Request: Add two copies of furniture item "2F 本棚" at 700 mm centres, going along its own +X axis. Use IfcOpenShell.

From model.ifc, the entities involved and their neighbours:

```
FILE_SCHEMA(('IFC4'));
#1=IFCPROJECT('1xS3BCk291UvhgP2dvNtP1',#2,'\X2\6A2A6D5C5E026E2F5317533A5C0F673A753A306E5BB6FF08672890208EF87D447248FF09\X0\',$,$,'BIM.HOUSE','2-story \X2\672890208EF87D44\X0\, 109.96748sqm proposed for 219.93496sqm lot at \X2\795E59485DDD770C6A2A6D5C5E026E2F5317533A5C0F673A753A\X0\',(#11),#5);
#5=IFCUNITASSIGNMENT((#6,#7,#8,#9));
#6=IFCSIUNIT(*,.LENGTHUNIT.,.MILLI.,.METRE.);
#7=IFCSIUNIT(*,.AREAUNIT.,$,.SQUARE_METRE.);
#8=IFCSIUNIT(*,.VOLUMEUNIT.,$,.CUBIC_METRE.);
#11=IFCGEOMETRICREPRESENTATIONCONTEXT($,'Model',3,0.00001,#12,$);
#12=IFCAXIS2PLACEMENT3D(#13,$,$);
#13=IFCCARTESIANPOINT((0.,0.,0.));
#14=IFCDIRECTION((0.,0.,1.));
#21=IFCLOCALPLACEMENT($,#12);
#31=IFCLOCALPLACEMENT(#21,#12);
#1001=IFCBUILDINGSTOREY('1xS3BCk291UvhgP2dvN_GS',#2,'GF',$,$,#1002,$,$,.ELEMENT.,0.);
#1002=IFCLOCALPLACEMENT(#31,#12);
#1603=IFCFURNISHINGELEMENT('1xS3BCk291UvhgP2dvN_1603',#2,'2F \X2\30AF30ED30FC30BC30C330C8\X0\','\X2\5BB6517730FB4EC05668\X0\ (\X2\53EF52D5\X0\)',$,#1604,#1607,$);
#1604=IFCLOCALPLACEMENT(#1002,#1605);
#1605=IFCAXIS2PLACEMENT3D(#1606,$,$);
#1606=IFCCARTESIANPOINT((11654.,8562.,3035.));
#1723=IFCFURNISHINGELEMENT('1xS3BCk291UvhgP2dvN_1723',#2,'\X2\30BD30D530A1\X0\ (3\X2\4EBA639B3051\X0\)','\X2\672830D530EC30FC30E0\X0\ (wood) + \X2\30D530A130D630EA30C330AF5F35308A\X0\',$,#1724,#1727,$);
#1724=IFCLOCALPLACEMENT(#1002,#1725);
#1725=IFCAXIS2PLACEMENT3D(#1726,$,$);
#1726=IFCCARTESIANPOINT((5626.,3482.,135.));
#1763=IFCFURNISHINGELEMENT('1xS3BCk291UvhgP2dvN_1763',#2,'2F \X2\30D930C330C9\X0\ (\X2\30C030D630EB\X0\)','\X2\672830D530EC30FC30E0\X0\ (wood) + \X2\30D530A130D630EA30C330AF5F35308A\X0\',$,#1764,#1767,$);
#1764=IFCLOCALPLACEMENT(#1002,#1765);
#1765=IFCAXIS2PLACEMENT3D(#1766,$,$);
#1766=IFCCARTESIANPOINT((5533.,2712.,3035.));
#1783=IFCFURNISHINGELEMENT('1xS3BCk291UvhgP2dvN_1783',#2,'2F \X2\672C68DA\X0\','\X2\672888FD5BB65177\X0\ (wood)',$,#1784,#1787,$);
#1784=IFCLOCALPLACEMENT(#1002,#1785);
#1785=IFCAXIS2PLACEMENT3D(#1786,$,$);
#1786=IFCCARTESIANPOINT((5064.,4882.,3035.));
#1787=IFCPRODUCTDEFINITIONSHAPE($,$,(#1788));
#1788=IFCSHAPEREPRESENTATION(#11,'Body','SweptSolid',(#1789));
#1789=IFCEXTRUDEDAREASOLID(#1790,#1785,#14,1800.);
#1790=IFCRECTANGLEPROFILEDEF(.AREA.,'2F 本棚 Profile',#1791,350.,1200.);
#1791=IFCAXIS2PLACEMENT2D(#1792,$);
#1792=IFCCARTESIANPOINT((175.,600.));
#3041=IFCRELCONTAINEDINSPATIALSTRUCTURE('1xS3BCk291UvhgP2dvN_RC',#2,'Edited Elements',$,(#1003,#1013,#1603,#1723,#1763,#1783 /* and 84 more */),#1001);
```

```python
import ifcopenshell
import ifcopenshell.api.geometry
import ifcopenshell.api.root
import ifcopenshell.util.element
import ifcopenshell.util.placement

model = ifcopenshell.open("model.ifc")


def reuse_history(source, copy):
    """copy_class also copies each property set's owner history, people and application; keep the originals."""
    for rel in copy.IsDefinedBy:
        if rel.is_a("IfcRelDefinesByProperties") and (history := rel.RelatingPropertyDefinition.OwnerHistory):
            rel.RelatingPropertyDefinition.OwnerHistory = source.OwnerHistory
            ifcopenshell.util.element.remove_deep2(model, history)


source = model.by_guid("1xS3BCk291UvhgP2dvN_1783")
base = ifcopenshell.util.placement.get_local_placement(source.ObjectPlacement)
step = base[:3, 0] * 700.0

for i in range(1, 3):
    copy = ifcopenshell.api.root.copy_class(model, product=source)
    copy.Representation = ifcopenshell.util.element.copy_deep(
        model, source.Representation, exclude=["IfcGeometricRepresentationContext", "IfcRepresentationMap"]
    )
    reuse_history(source, copy)
    matrix = base.copy()
    matrix[:3, 3] += i * step
    print("added at", matrix[:3, 3].round(3) + 0.0)
    ifcopenshell.api.geometry.edit_object_placement(model, product=copy, matrix=matrix, is_si=False)

model.write("model_edited.ifc")
```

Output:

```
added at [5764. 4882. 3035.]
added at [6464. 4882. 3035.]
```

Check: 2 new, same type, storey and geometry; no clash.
